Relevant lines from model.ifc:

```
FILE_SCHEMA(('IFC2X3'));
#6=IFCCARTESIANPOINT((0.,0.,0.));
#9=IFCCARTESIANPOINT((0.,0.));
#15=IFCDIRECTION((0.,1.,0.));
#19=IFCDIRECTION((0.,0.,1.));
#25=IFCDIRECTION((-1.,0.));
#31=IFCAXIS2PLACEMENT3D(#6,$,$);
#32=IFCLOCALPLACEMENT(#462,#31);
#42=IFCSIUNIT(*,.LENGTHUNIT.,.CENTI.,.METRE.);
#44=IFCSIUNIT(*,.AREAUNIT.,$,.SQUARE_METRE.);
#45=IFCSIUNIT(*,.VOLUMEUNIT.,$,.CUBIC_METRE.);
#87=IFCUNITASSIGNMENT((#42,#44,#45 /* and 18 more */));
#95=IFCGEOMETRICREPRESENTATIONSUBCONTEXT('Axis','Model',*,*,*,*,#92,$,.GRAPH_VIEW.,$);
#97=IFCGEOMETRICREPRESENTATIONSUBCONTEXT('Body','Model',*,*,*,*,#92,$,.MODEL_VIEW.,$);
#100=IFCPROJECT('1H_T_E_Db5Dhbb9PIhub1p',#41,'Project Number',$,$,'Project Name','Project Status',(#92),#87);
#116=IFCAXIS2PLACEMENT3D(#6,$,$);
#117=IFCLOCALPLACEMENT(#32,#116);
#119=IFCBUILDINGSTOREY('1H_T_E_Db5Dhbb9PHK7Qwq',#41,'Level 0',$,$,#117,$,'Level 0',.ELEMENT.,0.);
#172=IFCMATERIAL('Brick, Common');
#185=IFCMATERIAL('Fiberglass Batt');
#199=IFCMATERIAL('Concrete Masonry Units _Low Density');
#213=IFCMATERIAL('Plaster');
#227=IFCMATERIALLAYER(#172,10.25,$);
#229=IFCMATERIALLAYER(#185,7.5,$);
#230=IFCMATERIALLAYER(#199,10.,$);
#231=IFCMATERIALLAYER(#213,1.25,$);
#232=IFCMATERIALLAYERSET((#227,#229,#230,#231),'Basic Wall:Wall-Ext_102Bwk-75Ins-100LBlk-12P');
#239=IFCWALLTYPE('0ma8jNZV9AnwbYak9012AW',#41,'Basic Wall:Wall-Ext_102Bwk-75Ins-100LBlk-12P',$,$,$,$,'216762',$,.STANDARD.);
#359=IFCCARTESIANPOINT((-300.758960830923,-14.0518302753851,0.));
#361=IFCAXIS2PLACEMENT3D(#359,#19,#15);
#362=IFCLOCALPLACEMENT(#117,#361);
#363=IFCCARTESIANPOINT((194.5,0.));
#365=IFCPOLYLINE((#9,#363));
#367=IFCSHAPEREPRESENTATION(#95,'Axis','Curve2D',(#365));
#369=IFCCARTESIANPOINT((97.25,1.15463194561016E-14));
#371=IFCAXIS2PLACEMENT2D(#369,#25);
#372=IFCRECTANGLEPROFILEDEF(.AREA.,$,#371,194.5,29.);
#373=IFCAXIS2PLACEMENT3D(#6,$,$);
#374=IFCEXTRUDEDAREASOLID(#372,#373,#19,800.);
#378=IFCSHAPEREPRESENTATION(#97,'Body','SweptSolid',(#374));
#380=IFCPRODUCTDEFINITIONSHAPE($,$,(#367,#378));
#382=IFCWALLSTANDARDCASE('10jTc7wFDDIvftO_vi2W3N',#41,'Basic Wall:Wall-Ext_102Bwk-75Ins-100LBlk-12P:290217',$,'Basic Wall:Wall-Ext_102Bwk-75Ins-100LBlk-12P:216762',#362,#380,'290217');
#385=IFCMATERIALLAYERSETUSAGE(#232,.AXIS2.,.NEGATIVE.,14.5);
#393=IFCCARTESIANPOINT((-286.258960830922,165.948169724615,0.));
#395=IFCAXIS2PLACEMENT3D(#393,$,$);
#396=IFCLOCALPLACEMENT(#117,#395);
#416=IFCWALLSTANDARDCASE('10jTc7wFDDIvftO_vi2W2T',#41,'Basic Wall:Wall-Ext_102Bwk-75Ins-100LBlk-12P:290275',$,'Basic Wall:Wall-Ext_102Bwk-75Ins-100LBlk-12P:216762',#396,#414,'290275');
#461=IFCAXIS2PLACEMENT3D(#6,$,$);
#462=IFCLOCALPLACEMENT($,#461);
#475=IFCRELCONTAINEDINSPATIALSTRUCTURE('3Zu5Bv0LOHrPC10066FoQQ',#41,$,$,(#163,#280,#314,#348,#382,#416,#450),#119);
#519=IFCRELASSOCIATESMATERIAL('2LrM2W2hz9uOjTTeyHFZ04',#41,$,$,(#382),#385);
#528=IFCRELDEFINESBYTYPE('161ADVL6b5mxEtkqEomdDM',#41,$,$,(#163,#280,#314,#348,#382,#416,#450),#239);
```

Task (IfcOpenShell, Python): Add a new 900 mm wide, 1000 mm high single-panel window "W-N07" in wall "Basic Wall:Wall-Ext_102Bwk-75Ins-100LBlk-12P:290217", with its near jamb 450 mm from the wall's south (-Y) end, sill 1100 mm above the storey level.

```python
import numpy as np
import ifcopenshell
import ifcopenshell.api.feature
import ifcopenshell.api.geometry
import ifcopenshell.api.root
import ifcopenshell.api.spatial
import ifcopenshell.api.type
import ifcopenshell.geom
import ifcopenshell.util.element
import ifcopenshell.util.placement
import ifcopenshell.util.representation
import ifcopenshell.util.shape
import ifcopenshell.util.unit

model = ifcopenshell.open("model.ifc")
unit_scale = ifcopenshell.util.unit.calculate_unit_scale(model)
settings = ifcopenshell.geom.settings()


def volume(element):
    """Net volume in cubic metres, openings subtracted."""
    shape = ifcopenshell.geom.create_shape(settings, element)
    return ifcopenshell.util.shape.get_volume(shape.geometry)


wall = model.by_id(382)
storey = ifcopenshell.util.element.get_container(wall, ifc_class="IfcBuildingStorey")
context = ifcopenshell.util.representation.get_context(model, "Model", "Body", "MODEL_VIEW")
before = volume(wall)

width, height, from_end, sill = 0.9, 1, 0.45, 1.1  # metres

# The wall runs along its own X axis, and the end named is its -X end.
wall_shape = ifcopenshell.geom.create_shape(settings, wall)
x, y, z = ifcopenshell.util.shape.get_vertices(wall_shape.geometry).T
start = x.min() + from_end
face, thickness = float(y.min()), float(y.max() - y.min())
wall_matrix = ifcopenshell.util.placement.get_local_placement(wall.ObjectPlacement)
level = ifcopenshell.util.placement.get_local_placement(storey.ObjectPlacement)[2, 3]


def in_wall(x, y):
    """Placement at x, y metres in the wall's axes, at sill height."""
    matrix = wall_matrix.copy()
    matrix[:, 3] = wall_matrix @ np.array([x / unit_scale, y / unit_scale, 0.0, 1.0])
    matrix[2, 3] = level + sill / unit_scale
    return matrix


# Opening: a box that overshoots both wall faces by 50 mm.
opening = ifcopenshell.api.root.create_entity(model, ifc_class="IfcOpeningElement")
box = ifcopenshell.api.geometry.add_wall_representation(
    model, context=context, length=width, height=height, thickness=thickness + 0.1
)
ifcopenshell.api.geometry.assign_representation(model, product=opening, representation=box)
ifcopenshell.api.geometry.edit_object_placement(model, product=opening, matrix=in_wall(start, face - 0.05), is_si=False)
ifcopenshell.api.feature.add_feature(model, feature=opening, element=wall)

window = ifcopenshell.api.root.create_entity(model, ifc_class="IfcWindow", name="W-N07")
window.OverallWidth, window.OverallHeight = width / unit_scale, height / unit_scale
body = ifcopenshell.api.geometry.add_window_representation(
    model,
    context=context,
    overall_width=window.OverallWidth,
    overall_height=window.OverallHeight,
    partition_type="SINGLE_PANEL",
)
ifcopenshell.api.geometry.assign_representation(model, product=window, representation=body)
ifcopenshell.api.spatial.assign_container(model, products=[window], relating_structure=storey)
fills = ifcopenshell.api.feature.add_filling(model, opening=opening, element=window)
fills.OwnerHistory = window.OwnerHistory  # required in IFC2X3

# IFC2X3 keeps the operation on the window style.
style = ifcopenshell.api.root.create_entity(model, ifc_class="IfcWindowStyle", name="W-N07")
style.OperationType, style.ConstructionType = "SINGLE_PANEL", "NOTDEFINED"
style.ParameterTakesPrecedence = style.Sizeable = False
ifcopenshell.api.type.assign_type(model, related_objects=[window], relating_type=style)

# Centre the window in the wall's thickness.
ifcopenshell.api.geometry.edit_object_placement(model, product=window, matrix=in_wall(start, face), is_si=False)
window_shape = ifcopenshell.geom.create_shape(settings, window)
depth = ifcopenshell.util.shape.get_vertices(window_shape.geometry)[:, 1]
offset = face + thickness / 2 - (depth.min() + depth.max()) / 2
ifcopenshell.api.geometry.edit_object_placement(model, product=window, matrix=in_wall(start, offset), is_si=False)

after = volume(wall)

print(f"wall volume {before:.3f} -> {after:.3f} m3")

model.write("model_rev.ifc")
```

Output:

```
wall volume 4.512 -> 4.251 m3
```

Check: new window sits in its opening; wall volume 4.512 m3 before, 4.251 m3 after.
